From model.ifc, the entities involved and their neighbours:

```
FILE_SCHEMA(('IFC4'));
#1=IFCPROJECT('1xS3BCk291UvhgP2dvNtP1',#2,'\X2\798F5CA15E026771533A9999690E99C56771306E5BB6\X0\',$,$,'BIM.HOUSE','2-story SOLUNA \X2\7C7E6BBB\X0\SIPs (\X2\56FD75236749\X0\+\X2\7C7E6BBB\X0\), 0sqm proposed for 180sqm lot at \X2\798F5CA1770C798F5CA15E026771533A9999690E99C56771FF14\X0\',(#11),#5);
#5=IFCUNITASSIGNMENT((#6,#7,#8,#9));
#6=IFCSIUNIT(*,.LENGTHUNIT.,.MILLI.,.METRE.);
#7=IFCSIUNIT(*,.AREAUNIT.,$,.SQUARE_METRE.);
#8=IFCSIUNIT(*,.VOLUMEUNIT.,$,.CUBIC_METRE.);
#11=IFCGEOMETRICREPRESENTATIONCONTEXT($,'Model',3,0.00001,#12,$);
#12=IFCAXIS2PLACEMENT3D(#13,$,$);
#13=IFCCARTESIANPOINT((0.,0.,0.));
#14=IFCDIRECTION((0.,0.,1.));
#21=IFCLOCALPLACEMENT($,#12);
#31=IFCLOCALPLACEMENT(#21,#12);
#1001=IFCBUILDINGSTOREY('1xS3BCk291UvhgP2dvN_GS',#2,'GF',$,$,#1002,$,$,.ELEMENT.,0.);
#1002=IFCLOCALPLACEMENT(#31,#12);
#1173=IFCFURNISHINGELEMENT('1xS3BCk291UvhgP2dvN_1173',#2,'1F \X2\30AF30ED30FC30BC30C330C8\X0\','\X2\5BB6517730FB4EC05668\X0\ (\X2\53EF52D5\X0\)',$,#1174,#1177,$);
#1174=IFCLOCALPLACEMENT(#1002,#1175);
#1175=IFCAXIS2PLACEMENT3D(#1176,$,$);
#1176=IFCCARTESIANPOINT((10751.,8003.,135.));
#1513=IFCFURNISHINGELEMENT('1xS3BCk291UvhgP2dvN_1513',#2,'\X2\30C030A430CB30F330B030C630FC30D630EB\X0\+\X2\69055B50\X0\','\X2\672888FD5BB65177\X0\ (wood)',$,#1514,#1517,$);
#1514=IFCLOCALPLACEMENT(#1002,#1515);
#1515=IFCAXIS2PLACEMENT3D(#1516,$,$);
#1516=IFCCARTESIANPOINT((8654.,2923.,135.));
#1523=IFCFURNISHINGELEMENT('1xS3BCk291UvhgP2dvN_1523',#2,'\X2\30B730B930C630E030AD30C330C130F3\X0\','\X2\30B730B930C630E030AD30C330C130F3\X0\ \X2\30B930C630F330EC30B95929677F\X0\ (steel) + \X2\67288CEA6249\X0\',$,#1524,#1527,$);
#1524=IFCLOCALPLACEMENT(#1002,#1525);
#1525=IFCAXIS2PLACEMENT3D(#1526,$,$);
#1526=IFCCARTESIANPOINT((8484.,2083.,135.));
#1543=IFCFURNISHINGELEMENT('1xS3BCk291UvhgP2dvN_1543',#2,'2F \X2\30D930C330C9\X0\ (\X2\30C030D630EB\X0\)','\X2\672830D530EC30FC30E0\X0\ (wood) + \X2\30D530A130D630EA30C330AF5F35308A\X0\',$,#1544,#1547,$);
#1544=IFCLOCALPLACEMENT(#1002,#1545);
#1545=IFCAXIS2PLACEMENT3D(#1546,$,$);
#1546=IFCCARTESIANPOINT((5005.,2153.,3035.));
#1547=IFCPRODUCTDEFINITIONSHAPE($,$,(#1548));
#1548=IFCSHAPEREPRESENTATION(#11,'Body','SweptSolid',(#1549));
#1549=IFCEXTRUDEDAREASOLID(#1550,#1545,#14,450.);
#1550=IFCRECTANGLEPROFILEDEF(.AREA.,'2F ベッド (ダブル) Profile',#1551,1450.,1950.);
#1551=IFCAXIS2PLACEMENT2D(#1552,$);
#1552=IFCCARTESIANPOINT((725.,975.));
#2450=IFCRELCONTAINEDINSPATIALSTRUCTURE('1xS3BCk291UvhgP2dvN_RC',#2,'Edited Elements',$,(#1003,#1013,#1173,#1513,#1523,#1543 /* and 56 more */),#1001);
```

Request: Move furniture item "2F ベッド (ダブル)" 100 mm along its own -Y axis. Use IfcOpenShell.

```python
import ifcopenshell
import ifcopenshell.api.geometry
import ifcopenshell.util.placement
import ifcopenshell.util.unit

model = ifcopenshell.open("model.ifc")
unit_scale = ifcopenshell.util.unit.calculate_unit_scale(model)

item = model.by_guid("1xS3BCk291UvhgP2dvN_1543")
matrix = ifcopenshell.util.placement.get_local_placement(item.ObjectPlacement)
matrix[:3, 3] -= matrix[:3, 1] * 0.1 / unit_scale
ifcopenshell.api.geometry.edit_object_placement(model, product=item, matrix=matrix, is_si=False)

print(ifcopenshell.util.placement.get_local_placement(item.ObjectPlacement).round(3) + 0.0)

model.write("model_rev.ifc")
```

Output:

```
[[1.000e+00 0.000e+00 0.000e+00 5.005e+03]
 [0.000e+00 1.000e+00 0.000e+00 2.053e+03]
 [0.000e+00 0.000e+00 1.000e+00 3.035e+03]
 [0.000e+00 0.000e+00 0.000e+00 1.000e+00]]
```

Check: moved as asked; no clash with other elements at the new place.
